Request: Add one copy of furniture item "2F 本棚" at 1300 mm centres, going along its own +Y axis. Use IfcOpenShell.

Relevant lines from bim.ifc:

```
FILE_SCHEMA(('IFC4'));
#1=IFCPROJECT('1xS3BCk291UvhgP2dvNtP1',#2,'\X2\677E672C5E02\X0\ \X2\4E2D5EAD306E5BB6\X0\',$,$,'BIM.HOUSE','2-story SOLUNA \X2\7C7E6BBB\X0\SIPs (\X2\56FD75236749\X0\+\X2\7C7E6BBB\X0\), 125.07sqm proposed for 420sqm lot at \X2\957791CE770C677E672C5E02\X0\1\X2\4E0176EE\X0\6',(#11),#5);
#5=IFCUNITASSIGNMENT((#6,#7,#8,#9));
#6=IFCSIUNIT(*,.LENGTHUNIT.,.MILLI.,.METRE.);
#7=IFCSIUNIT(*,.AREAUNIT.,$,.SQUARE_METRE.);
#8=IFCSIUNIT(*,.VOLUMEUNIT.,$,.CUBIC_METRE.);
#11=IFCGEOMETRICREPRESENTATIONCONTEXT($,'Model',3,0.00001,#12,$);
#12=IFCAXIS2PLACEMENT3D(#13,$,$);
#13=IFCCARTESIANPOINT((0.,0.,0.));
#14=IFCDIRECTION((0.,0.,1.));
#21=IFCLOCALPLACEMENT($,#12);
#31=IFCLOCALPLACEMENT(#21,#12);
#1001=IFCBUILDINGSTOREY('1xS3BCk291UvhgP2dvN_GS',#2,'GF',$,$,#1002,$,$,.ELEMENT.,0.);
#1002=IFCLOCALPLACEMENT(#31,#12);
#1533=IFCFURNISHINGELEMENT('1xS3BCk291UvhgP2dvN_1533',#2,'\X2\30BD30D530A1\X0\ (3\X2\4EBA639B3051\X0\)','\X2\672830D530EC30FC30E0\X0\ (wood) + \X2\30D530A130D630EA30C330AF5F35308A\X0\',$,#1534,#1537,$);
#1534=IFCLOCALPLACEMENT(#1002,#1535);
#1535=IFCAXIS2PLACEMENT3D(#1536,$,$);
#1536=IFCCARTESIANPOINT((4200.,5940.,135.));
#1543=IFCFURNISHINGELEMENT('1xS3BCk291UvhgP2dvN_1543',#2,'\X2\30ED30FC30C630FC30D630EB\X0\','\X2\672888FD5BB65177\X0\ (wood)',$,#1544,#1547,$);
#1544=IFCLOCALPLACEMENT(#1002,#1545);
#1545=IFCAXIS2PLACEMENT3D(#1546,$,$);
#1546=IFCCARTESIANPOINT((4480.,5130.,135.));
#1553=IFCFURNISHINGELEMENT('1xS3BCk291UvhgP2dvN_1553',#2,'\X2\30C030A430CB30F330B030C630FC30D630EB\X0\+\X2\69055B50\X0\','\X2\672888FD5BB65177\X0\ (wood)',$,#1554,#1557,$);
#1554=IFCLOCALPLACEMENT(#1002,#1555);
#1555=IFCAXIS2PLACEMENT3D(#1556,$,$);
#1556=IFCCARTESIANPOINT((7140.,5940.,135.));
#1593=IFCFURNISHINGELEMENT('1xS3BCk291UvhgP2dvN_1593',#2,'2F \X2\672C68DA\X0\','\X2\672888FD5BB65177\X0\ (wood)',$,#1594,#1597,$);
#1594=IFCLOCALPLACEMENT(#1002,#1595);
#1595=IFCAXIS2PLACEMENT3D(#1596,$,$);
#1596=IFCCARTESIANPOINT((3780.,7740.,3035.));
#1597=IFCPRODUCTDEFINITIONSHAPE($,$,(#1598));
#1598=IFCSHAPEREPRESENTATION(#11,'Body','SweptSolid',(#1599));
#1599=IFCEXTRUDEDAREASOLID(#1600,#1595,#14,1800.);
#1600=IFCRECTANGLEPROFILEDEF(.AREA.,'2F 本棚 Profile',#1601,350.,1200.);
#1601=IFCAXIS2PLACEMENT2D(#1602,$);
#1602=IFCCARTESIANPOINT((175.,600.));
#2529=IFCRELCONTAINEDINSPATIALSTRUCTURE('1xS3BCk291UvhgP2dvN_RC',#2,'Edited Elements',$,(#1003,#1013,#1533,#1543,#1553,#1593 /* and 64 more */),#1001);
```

```python
import ifcopenshell
import ifcopenshell.api.geometry
import ifcopenshell.api.root
import ifcopenshell.util.element
import ifcopenshell.util.placement

model = ifcopenshell.open("bim.ifc")


def reuse_history(source, copy):
    """copy_class also copies each property set's owner history, people and application; keep the originals."""
    for rel in copy.IsDefinedBy:
        if rel.is_a("IfcRelDefinesByProperties") and (history := rel.RelatingPropertyDefinition.OwnerHistory):
            rel.RelatingPropertyDefinition.OwnerHistory = source.OwnerHistory
            ifcopenshell.util.element.remove_deep2(model, history)


source = model.by_guid("1xS3BCk291UvhgP2dvN_1593")
base = ifcopenshell.util.placement.get_local_placement(source.ObjectPlacement)
step = base[:3, 1] * 1300.0

for i in range(1, 2):
    copy = ifcopenshell.api.root.copy_class(model, product=source)
    copy.Representation = ifcopenshell.util.element.copy_deep(
        model, source.Representation, exclude=["IfcGeometricRepresentationContext", "IfcRepresentationMap"]
    )
    reuse_history(source, copy)
    matrix = base.copy()
    matrix[:3, 3] += i * step
    print("added at", matrix[:3, 3].round(3) + 0.0)
    ifcopenshell.api.geometry.edit_object_placement(model, product=copy, matrix=matrix, is_si=False)

model.write("bim_rev.ifc")
```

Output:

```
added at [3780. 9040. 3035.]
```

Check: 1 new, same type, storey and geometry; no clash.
